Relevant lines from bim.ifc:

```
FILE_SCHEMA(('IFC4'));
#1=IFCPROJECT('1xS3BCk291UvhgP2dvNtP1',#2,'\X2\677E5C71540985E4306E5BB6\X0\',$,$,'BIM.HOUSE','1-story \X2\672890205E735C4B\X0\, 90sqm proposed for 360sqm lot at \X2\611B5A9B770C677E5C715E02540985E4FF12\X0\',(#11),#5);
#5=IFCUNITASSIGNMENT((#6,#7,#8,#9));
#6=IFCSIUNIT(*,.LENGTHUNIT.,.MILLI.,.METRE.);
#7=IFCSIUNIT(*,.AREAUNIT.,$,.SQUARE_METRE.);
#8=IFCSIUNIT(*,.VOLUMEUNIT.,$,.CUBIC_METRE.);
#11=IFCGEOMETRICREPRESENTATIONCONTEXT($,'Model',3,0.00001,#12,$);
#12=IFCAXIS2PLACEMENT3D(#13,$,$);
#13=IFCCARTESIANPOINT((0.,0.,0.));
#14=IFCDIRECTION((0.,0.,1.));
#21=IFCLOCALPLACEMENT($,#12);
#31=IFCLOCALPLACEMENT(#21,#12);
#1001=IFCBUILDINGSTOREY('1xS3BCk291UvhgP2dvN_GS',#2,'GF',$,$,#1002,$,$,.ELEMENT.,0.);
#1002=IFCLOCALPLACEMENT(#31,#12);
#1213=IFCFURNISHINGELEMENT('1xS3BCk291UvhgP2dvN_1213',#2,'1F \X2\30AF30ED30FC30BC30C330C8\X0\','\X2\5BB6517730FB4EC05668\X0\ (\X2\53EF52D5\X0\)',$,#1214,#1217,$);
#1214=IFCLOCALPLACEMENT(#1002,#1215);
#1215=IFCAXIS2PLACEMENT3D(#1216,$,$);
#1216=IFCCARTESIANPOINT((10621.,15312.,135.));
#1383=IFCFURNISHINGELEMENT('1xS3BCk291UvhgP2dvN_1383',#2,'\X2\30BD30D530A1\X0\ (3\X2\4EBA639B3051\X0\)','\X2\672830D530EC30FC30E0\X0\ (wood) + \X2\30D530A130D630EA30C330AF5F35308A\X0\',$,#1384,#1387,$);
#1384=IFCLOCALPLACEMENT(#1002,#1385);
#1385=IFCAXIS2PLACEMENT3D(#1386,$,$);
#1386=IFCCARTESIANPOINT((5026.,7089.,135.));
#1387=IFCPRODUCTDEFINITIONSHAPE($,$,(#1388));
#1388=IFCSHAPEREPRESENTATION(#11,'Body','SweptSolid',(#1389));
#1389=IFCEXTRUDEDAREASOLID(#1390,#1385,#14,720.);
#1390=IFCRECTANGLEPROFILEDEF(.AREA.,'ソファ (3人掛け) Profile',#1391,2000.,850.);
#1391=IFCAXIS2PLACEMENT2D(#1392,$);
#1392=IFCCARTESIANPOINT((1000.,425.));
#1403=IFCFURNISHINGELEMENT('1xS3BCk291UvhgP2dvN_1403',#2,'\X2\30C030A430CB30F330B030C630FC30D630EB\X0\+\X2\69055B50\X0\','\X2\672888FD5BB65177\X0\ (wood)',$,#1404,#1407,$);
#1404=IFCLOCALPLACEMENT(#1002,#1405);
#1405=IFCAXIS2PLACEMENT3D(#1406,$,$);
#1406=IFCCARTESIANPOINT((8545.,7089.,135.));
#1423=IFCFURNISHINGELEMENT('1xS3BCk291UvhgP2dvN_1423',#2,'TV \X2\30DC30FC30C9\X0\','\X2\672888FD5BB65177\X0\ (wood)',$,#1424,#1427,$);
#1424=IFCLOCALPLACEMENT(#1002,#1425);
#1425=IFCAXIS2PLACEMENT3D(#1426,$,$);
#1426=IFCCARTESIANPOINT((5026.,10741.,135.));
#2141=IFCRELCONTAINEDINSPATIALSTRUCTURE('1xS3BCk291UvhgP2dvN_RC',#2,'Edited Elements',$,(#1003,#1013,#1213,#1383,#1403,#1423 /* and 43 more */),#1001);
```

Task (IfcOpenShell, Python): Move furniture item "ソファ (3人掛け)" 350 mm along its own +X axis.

```python
import ifcopenshell
import ifcopenshell.api.geometry
import ifcopenshell.util.placement
import ifcopenshell.util.unit

model = ifcopenshell.open("bim.ifc")
unit_scale = ifcopenshell.util.unit.calculate_unit_scale(model)

item = model.by_id(1383)
matrix = ifcopenshell.util.placement.get_local_placement(item.ObjectPlacement)
matrix[:3, 3] += matrix[:3, 0] * 0.35 / unit_scale
ifcopenshell.api.geometry.edit_object_placement(model, product=item, matrix=matrix, is_si=False)

print(ifcopenshell.util.placement.get_local_placement(item.ObjectPlacement).round(3) + 0.0)

model.write("bim_edited.ifc")
```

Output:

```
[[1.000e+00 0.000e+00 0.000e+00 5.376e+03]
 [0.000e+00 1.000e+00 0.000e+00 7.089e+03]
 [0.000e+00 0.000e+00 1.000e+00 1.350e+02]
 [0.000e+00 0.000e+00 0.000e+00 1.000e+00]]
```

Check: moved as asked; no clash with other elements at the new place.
